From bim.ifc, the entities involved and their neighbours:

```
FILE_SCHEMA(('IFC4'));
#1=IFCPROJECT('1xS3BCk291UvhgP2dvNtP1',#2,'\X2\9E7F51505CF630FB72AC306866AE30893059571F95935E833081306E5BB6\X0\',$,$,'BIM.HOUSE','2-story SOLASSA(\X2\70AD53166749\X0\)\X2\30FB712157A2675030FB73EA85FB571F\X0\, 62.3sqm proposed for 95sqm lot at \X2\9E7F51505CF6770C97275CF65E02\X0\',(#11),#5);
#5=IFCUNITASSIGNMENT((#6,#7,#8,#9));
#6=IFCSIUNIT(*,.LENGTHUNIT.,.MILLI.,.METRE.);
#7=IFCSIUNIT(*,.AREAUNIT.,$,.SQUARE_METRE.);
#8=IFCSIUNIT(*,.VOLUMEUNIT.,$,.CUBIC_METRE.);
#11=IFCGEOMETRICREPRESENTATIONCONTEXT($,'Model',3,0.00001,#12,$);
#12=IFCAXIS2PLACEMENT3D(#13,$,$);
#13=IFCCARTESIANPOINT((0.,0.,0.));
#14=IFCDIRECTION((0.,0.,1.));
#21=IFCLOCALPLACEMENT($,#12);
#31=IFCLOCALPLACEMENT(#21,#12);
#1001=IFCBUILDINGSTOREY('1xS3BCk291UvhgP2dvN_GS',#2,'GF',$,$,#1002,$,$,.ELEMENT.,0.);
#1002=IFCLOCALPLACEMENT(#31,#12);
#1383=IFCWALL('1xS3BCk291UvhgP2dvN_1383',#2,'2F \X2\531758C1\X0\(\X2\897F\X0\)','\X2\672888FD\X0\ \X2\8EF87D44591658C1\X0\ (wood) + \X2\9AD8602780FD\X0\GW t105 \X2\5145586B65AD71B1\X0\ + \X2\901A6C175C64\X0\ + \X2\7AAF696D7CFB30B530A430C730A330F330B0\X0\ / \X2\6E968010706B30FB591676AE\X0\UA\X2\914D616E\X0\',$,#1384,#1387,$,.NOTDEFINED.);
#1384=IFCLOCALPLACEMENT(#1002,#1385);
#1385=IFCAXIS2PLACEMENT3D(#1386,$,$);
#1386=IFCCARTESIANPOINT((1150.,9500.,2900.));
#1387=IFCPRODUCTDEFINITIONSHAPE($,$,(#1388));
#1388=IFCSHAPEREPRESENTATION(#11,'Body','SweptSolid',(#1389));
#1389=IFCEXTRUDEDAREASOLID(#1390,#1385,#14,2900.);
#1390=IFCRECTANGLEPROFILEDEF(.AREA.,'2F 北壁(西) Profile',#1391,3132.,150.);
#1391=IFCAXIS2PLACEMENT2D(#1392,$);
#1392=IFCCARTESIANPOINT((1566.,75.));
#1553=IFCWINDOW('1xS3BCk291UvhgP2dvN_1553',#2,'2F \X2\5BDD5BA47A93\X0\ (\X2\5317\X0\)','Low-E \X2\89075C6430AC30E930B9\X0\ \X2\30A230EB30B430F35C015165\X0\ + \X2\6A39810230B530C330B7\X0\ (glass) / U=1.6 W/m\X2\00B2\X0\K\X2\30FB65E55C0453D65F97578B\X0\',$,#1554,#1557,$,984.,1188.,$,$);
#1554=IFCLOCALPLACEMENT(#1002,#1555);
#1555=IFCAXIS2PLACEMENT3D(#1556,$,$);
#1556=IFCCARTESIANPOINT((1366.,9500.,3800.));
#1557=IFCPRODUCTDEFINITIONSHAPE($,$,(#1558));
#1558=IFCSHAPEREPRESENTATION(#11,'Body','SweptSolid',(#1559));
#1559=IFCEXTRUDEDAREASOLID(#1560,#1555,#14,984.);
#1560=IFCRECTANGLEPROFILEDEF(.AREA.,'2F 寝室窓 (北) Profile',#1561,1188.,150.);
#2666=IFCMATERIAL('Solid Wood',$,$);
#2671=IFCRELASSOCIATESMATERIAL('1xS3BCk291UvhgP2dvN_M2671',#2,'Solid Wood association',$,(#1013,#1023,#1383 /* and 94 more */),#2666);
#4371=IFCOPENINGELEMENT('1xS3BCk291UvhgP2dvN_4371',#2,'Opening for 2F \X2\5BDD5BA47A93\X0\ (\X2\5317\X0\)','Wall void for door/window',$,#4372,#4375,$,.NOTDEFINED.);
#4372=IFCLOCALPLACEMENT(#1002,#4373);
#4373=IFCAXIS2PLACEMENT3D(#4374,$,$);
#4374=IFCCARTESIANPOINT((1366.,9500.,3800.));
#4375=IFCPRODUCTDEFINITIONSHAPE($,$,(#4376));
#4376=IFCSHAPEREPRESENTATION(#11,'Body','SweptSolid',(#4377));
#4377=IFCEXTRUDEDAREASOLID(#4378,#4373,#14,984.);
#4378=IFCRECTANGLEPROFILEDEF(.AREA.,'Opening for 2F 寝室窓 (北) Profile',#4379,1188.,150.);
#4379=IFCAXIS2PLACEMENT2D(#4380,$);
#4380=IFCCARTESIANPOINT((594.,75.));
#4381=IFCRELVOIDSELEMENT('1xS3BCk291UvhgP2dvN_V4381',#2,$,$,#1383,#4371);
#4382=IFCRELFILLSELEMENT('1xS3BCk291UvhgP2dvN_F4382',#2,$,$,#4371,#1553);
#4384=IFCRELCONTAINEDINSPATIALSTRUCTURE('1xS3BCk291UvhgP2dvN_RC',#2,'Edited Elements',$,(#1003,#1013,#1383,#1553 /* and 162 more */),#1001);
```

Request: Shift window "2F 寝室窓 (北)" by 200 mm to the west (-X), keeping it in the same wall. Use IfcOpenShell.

```python
import ifcopenshell
import ifcopenshell.api.geometry
import ifcopenshell.util.placement
import ifcopenshell.util.unit

model = ifcopenshell.open("bim.ifc")
unit_scale = ifcopenshell.util.unit.calculate_unit_scale(model)

window = model.by_guid("1xS3BCk291UvhgP2dvN_1553")
opening = window.FillsVoids[0].RelatingOpeningElement
wall = opening.VoidsElements[0].RelatingBuildingElement

wall_matrix = ifcopenshell.util.placement.get_local_placement(wall.ObjectPlacement)
shift = wall_matrix[:3, 0] * -0.2 / unit_scale
before = ifcopenshell.util.placement.get_local_placement(window.ObjectPlacement)[:3, 3].copy()

# The window is not placed relative to its opening, so move both.
for product in (opening, window):
    matrix = ifcopenshell.util.placement.get_local_placement(product.ObjectPlacement)
    matrix[:3, 3] += shift
    ifcopenshell.api.geometry.edit_object_placement(model, product=product, matrix=matrix, is_si=False)

after = ifcopenshell.util.placement.get_local_placement(window.ObjectPlacement)[:3, 3]
print("window moved by", (after - before).round(3) + 0.0)

model.write("bim_rev.ifc")
```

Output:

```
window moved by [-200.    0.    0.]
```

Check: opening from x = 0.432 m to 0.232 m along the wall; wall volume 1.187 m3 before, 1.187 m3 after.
